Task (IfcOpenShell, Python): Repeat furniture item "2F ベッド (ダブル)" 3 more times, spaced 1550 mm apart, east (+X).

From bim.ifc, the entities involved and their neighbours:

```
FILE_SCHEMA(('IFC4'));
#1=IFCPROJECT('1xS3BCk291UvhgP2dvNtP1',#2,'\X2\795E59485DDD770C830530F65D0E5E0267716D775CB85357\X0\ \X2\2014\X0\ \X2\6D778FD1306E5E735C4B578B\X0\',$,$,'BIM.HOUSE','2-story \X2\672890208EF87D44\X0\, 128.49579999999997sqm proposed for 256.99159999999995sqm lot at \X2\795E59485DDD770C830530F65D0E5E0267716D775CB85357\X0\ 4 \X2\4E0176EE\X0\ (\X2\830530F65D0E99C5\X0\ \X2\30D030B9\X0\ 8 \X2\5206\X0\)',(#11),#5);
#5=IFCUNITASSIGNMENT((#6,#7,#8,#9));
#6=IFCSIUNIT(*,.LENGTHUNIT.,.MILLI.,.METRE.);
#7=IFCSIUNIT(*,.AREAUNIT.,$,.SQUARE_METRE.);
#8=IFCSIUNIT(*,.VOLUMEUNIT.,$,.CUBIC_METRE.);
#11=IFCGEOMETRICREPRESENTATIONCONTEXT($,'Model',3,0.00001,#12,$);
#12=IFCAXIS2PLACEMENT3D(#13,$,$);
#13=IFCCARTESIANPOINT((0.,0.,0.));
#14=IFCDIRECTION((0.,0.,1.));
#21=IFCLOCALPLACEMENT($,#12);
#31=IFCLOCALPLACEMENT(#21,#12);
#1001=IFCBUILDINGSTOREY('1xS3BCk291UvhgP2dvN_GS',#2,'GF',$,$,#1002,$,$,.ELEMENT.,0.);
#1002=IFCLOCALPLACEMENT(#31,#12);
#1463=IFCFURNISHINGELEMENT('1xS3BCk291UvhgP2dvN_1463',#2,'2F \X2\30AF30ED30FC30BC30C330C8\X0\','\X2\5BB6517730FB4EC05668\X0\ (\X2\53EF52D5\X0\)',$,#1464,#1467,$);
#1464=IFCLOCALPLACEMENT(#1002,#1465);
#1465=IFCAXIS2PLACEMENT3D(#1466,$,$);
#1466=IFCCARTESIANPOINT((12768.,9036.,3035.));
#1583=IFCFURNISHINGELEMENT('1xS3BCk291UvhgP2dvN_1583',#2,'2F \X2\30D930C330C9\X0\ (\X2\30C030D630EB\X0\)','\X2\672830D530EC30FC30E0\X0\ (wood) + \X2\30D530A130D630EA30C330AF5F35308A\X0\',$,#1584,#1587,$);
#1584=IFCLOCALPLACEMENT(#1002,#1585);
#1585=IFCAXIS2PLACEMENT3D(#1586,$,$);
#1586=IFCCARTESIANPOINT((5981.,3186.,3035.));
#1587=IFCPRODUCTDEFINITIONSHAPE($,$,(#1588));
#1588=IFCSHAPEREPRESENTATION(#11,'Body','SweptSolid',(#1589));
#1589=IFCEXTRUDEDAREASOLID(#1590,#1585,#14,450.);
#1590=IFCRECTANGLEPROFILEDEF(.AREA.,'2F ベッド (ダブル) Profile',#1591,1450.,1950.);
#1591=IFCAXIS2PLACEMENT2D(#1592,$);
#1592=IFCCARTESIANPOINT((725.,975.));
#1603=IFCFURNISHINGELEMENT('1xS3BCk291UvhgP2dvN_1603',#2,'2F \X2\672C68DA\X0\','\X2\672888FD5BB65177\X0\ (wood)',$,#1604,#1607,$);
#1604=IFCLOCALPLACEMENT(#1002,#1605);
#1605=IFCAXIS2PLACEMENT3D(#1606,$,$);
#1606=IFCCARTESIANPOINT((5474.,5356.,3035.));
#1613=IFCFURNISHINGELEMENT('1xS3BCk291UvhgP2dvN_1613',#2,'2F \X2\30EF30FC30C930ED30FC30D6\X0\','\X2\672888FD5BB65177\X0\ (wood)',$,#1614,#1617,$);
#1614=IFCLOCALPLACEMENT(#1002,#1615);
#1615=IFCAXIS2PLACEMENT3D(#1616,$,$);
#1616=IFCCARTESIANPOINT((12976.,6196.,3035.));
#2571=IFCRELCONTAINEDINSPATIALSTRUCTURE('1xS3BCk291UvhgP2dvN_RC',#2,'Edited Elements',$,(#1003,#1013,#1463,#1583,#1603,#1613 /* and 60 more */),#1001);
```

```python
import numpy as np
import ifcopenshell
import ifcopenshell.api.geometry
import ifcopenshell.api.root
import ifcopenshell.util.element
import ifcopenshell.util.placement
import ifcopenshell.util.unit

model = ifcopenshell.open("bim.ifc")
unit_scale = ifcopenshell.util.unit.calculate_unit_scale(model)


def reuse_history(source, copy):
    """copy_class also copies each property set's owner history, people and application; keep the originals."""
    for rel in copy.IsDefinedBy:
        if rel.is_a("IfcRelDefinesByProperties") and (history := rel.RelatingPropertyDefinition.OwnerHistory):
            rel.RelatingPropertyDefinition.OwnerHistory = source.OwnerHistory
            ifcopenshell.util.element.remove_deep2(model, history)


source = model.by_id(1583)
base = ifcopenshell.util.placement.get_local_placement(source.ObjectPlacement)
step = np.array([1.0, 0.0, 0.0]) * 1.55 / unit_scale

for i in range(1, 4):
    copy = ifcopenshell.api.root.copy_class(model, product=source)
    copy.Representation = ifcopenshell.util.element.copy_deep(
        model, source.Representation, exclude=["IfcGeometricRepresentationContext", "IfcRepresentationMap"]
    )
    reuse_history(source, copy)
    matrix = base.copy()
    matrix[:3, 3] += i * step
    print("added at", matrix[:3, 3].round(3) + 0.0)
    ifcopenshell.api.geometry.edit_object_placement(model, product=copy, matrix=matrix, is_si=False)

model.write("bim_edited.ifc")
```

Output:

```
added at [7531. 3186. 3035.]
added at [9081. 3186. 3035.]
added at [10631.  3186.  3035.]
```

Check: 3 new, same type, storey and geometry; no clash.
